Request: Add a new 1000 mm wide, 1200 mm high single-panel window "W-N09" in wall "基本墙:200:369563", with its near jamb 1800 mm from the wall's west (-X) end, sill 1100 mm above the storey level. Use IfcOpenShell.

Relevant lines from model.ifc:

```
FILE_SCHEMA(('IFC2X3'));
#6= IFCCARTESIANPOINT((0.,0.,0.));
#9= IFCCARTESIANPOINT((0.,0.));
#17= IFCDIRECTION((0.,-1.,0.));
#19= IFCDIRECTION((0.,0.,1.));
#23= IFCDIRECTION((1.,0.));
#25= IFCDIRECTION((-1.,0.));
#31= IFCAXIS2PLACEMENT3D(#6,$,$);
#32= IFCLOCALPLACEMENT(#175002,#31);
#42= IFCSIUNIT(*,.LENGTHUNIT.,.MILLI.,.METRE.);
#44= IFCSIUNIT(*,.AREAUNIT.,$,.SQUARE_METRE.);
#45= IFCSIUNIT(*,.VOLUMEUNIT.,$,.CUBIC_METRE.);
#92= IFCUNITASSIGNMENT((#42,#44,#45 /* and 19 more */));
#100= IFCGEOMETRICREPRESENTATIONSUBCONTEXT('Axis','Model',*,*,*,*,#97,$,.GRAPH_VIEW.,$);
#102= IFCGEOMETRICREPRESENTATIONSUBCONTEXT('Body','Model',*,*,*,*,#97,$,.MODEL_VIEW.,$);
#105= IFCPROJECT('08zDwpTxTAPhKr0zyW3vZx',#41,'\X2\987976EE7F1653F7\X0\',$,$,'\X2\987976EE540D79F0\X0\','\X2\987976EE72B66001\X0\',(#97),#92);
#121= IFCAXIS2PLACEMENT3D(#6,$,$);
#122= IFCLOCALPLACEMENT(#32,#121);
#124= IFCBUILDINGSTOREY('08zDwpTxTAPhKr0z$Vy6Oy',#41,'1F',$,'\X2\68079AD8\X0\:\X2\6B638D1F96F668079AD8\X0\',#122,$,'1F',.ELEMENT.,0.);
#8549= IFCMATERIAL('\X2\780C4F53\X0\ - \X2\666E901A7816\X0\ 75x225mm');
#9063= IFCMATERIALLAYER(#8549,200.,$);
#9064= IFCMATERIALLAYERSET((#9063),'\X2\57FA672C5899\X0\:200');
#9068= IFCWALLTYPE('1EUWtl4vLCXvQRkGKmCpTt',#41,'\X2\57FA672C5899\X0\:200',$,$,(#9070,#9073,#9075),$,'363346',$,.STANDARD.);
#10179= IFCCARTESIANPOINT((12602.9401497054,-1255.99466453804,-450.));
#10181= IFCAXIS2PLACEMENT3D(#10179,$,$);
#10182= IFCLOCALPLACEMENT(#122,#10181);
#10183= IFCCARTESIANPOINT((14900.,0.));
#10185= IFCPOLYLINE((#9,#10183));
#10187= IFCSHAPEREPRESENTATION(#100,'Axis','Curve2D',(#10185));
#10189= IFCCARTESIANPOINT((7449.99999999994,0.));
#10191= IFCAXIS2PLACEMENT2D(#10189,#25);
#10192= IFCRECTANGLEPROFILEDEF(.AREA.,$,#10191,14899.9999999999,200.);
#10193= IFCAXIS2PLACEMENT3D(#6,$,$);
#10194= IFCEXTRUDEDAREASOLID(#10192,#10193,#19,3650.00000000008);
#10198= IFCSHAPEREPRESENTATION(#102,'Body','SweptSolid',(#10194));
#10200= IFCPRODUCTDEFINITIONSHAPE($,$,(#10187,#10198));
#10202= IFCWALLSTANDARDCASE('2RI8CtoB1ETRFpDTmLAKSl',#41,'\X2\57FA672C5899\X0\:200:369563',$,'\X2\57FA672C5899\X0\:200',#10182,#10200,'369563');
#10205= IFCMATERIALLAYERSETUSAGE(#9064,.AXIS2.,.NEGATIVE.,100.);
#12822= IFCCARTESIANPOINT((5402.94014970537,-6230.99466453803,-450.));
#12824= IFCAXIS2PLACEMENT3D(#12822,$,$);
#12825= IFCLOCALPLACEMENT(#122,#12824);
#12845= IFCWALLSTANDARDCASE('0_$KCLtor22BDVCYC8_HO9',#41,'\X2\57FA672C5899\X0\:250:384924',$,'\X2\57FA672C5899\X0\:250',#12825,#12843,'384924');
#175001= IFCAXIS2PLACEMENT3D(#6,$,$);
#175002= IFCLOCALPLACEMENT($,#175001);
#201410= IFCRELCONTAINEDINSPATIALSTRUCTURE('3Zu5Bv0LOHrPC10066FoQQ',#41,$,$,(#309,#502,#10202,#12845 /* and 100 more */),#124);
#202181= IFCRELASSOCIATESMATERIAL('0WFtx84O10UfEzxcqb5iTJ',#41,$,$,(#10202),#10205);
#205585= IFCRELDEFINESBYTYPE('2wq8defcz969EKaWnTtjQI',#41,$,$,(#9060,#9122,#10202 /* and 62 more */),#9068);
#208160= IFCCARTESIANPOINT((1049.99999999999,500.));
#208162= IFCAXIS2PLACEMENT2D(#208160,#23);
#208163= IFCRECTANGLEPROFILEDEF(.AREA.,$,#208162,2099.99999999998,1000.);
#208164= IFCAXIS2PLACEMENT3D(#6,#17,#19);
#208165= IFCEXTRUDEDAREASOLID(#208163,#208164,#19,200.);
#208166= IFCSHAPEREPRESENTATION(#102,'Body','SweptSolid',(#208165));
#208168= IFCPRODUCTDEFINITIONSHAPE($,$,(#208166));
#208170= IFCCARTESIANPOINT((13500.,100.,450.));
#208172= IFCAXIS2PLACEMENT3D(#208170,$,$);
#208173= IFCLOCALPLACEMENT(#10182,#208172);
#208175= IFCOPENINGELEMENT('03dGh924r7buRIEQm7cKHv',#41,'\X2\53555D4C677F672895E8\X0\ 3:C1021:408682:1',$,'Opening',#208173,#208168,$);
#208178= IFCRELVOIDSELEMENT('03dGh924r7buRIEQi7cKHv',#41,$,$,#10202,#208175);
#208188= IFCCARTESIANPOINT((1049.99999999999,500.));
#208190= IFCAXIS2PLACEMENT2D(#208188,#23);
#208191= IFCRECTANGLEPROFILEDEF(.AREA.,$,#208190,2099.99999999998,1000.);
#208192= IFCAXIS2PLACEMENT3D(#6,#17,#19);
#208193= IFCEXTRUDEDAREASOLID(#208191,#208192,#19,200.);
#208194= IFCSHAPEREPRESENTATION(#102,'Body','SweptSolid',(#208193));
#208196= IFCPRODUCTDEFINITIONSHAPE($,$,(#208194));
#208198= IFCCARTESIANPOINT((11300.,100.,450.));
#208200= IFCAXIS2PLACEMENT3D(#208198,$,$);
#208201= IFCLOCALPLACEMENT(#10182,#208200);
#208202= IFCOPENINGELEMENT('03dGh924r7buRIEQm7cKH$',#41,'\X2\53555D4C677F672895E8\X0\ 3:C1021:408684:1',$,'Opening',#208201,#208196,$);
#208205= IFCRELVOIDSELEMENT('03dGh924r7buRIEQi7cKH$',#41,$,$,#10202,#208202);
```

```python
import numpy as np
import ifcopenshell
import ifcopenshell.api.feature
import ifcopenshell.api.geometry
import ifcopenshell.api.root
import ifcopenshell.api.spatial
import ifcopenshell.api.type
import ifcopenshell.geom
import ifcopenshell.util.element
import ifcopenshell.util.placement
import ifcopenshell.util.representation
import ifcopenshell.util.shape
import ifcopenshell.util.unit

model = ifcopenshell.open("model.ifc")
unit_scale = ifcopenshell.util.unit.calculate_unit_scale(model)
settings = ifcopenshell.geom.settings()


def volume(element):
    """Net volume in cubic metres, openings subtracted."""
    shape = ifcopenshell.geom.create_shape(settings, element)
    return ifcopenshell.util.shape.get_volume(shape.geometry)


wall = model.by_id(10202)
storey = ifcopenshell.util.element.get_container(wall, ifc_class="IfcBuildingStorey")
context = ifcopenshell.util.representation.get_context(model, "Model", "Body", "MODEL_VIEW")
before = volume(wall)

width, height, from_end, sill = 1, 1.2, 1.8, 1.1  # metres

# The wall runs along its own X axis, and the end named is its -X end.
wall_shape = ifcopenshell.geom.create_shape(settings, wall)
x, y, z = ifcopenshell.util.shape.get_vertices(wall_shape.geometry).T
start = x.min() + from_end
face, thickness = float(y.min()), float(y.max() - y.min())
wall_matrix = ifcopenshell.util.placement.get_local_placement(wall.ObjectPlacement)
level = ifcopenshell.util.placement.get_local_placement(storey.ObjectPlacement)[2, 3]


def in_wall(x, y):
    """Placement at x, y metres in the wall's axes, at sill height."""
    matrix = wall_matrix.copy()
    matrix[:, 3] = wall_matrix @ np.array([x / unit_scale, y / unit_scale, 0.0, 1.0])
    matrix[2, 3] = level + sill / unit_scale
    return matrix


# Opening: a box that overshoots both wall faces by 50 mm.
opening = ifcopenshell.api.root.create_entity(model, ifc_class="IfcOpeningElement")
box = ifcopenshell.api.geometry.add_wall_representation(
    model, context=context, length=width, height=height, thickness=thickness + 0.1
)
ifcopenshell.api.geometry.assign_representation(model, product=opening, representation=box)
ifcopenshell.api.geometry.edit_object_placement(model, product=opening, matrix=in_wall(start, face - 0.05), is_si=False)
ifcopenshell.api.feature.add_feature(model, feature=opening, element=wall)

window = ifcopenshell.api.root.create_entity(model, ifc_class="IfcWindow", name="W-N09")
window.OverallWidth, window.OverallHeight = width / unit_scale, height / unit_scale
body = ifcopenshell.api.geometry.add_window_representation(
    model,
    context=context,
    overall_width=window.OverallWidth,
    overall_height=window.OverallHeight,
    partition_type="SINGLE_PANEL",
)
ifcopenshell.api.geometry.assign_representation(model, product=window, representation=body)
ifcopenshell.api.spatial.assign_container(model, products=[window], relating_structure=storey)
fills = ifcopenshell.api.feature.add_filling(model, opening=opening, element=window)
fills.OwnerHistory = window.OwnerHistory  # required in IFC2X3

# IFC2X3 keeps the operation on the window style.
style = ifcopenshell.api.root.create_entity(model, ifc_class="IfcWindowStyle", name="W-N09")
style.OperationType, style.ConstructionType = "SINGLE_PANEL", "NOTDEFINED"
style.ParameterTakesPrecedence = style.Sizeable = False
ifcopenshell.api.type.assign_type(model, related_objects=[window], relating_type=style)

# Centre the window in the wall's thickness.
ifcopenshell.api.geometry.edit_object_placement(model, product=window, matrix=in_wall(start, face), is_si=False)
window_shape = ifcopenshell.geom.create_shape(settings, window)
depth = ifcopenshell.util.shape.get_vertices(window_shape.geometry)[:, 1]
offset = face + thickness / 2 - (depth.min() + depth.max()) / 2
ifcopenshell.api.geometry.edit_object_placement(model, product=window, matrix=in_wall(start, offset), is_si=False)

after = volume(wall)

print(f"wall volume {before:.3f} -> {after:.3f} m3")

model.write("model_updated.ifc")
```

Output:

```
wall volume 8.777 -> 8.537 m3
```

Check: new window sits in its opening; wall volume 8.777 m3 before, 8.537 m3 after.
